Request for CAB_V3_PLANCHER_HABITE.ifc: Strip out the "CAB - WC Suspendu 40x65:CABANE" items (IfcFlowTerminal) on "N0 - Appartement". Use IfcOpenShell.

First a look at what the model holds.

```python
import ifcopenshell
import ifcopenshell.util.element

model = ifcopenshell.open("CAB_V3_PLANCHER_HABITE.ifc")
print(model.schema)
storey = next(s for s in model.by_type("IfcBuildingStorey") if s.Name == "N0 - Appartement")
terminals = [e for e in ifcopenshell.util.element.get_decomposition(storey) if e.is_a("IfcFlowTerminal")]
seen = {}
for e in terminals:
    element_type = ifcopenshell.util.element.get_type(e)
    name = element_type.Name if element_type not in (None, e) else None
    seen[name] = seen.get(name, 0) + 1
for name, count in sorted(seen.items(), key=str):
    print(count, "x", name)
```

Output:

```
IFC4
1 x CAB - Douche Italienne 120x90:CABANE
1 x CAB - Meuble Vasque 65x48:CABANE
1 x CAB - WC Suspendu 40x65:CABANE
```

```python
import ifcopenshell
import ifcopenshell.api.root
import ifcopenshell.util.element

model = ifcopenshell.open("CAB_V3_PLANCHER_HABITE.ifc")

storey = next(s for s in model.by_type("IfcBuildingStorey") if s.Name == "N0 - Appartement")
terminals = [e for e in ifcopenshell.util.element.get_decomposition(storey) if e.is_a("IfcFlowTerminal")]
targets = [e for e in terminals if (t := ifcopenshell.util.element.get_type(e)) not in (None, e) and t.Name == "CAB - WC Suspendu 40x65:CABANE"]

for e in targets:
    ifcopenshell.api.root.remove_product(model, product=e)
print(len(targets), "removed")

model.write("CAB_V3_PLANCHER_HABITE_v2.ifc")
```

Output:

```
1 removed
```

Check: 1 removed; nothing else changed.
